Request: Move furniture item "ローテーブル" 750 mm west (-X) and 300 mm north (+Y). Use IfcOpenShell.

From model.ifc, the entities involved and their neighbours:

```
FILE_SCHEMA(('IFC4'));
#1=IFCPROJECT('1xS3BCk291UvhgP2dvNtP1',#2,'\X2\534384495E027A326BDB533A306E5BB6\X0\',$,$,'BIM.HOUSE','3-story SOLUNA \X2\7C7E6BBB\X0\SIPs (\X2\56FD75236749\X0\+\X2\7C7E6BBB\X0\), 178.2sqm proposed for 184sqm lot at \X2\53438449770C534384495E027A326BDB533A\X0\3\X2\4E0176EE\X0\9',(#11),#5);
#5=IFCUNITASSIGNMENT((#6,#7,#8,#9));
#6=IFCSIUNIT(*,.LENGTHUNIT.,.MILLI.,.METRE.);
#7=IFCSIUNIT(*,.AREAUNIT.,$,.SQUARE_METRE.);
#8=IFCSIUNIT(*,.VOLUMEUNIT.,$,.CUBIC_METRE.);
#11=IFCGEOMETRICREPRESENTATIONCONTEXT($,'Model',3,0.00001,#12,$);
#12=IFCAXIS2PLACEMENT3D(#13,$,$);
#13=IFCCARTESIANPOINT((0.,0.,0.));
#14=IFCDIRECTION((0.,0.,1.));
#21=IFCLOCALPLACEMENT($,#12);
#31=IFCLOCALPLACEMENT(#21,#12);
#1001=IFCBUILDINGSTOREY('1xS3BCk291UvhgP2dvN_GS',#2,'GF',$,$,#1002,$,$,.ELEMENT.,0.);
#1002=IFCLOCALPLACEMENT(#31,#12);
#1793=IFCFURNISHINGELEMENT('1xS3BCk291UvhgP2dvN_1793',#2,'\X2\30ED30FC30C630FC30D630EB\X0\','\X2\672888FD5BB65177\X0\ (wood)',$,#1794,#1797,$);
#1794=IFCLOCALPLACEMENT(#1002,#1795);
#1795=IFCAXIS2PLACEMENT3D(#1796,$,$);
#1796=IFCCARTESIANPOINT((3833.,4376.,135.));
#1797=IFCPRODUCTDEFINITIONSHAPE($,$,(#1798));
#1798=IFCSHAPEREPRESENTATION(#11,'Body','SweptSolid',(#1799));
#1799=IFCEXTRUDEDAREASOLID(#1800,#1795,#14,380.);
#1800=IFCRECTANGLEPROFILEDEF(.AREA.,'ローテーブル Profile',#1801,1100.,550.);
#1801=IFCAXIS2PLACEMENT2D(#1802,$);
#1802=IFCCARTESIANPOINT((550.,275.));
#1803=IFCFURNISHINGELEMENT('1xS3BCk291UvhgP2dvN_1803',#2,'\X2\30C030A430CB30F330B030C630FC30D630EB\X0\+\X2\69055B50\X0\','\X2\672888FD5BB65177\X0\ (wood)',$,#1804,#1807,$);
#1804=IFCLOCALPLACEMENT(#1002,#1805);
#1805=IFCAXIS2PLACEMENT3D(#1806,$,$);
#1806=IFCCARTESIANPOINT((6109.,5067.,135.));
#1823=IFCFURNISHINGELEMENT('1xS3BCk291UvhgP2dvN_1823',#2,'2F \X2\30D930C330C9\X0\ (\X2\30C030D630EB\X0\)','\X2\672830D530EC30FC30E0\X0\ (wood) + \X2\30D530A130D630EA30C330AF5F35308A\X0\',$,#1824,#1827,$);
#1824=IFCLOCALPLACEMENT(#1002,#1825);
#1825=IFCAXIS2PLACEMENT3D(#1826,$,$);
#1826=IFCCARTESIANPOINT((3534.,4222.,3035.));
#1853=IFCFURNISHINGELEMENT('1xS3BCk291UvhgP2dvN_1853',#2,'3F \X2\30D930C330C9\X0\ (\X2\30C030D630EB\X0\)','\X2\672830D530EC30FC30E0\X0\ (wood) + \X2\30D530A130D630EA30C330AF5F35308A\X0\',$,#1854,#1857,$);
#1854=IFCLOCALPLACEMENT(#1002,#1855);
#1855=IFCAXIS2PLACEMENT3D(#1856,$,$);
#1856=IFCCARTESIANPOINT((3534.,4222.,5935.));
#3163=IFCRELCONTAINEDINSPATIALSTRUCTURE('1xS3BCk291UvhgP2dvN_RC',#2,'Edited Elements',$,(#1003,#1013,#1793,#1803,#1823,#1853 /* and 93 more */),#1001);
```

```python
import ifcopenshell
import ifcopenshell.api.geometry
import ifcopenshell.util.placement
import ifcopenshell.util.unit

model = ifcopenshell.open("model.ifc")
unit_scale = ifcopenshell.util.unit.calculate_unit_scale(model)

item = model.by_guid("1xS3BCk291UvhgP2dvN_1793")
matrix = ifcopenshell.util.placement.get_local_placement(item.ObjectPlacement)
matrix[0, 3] -= 0.75 / unit_scale
matrix[1, 3] += 0.3 / unit_scale
ifcopenshell.api.geometry.edit_object_placement(model, product=item, matrix=matrix, is_si=False)

print(ifcopenshell.util.placement.get_local_placement(item.ObjectPlacement).round(3) + 0.0)

model.write("model_rev.ifc")
```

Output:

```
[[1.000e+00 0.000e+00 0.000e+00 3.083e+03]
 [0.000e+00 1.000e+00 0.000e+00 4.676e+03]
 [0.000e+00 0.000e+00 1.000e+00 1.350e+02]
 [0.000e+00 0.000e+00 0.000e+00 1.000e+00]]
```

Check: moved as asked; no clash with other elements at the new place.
